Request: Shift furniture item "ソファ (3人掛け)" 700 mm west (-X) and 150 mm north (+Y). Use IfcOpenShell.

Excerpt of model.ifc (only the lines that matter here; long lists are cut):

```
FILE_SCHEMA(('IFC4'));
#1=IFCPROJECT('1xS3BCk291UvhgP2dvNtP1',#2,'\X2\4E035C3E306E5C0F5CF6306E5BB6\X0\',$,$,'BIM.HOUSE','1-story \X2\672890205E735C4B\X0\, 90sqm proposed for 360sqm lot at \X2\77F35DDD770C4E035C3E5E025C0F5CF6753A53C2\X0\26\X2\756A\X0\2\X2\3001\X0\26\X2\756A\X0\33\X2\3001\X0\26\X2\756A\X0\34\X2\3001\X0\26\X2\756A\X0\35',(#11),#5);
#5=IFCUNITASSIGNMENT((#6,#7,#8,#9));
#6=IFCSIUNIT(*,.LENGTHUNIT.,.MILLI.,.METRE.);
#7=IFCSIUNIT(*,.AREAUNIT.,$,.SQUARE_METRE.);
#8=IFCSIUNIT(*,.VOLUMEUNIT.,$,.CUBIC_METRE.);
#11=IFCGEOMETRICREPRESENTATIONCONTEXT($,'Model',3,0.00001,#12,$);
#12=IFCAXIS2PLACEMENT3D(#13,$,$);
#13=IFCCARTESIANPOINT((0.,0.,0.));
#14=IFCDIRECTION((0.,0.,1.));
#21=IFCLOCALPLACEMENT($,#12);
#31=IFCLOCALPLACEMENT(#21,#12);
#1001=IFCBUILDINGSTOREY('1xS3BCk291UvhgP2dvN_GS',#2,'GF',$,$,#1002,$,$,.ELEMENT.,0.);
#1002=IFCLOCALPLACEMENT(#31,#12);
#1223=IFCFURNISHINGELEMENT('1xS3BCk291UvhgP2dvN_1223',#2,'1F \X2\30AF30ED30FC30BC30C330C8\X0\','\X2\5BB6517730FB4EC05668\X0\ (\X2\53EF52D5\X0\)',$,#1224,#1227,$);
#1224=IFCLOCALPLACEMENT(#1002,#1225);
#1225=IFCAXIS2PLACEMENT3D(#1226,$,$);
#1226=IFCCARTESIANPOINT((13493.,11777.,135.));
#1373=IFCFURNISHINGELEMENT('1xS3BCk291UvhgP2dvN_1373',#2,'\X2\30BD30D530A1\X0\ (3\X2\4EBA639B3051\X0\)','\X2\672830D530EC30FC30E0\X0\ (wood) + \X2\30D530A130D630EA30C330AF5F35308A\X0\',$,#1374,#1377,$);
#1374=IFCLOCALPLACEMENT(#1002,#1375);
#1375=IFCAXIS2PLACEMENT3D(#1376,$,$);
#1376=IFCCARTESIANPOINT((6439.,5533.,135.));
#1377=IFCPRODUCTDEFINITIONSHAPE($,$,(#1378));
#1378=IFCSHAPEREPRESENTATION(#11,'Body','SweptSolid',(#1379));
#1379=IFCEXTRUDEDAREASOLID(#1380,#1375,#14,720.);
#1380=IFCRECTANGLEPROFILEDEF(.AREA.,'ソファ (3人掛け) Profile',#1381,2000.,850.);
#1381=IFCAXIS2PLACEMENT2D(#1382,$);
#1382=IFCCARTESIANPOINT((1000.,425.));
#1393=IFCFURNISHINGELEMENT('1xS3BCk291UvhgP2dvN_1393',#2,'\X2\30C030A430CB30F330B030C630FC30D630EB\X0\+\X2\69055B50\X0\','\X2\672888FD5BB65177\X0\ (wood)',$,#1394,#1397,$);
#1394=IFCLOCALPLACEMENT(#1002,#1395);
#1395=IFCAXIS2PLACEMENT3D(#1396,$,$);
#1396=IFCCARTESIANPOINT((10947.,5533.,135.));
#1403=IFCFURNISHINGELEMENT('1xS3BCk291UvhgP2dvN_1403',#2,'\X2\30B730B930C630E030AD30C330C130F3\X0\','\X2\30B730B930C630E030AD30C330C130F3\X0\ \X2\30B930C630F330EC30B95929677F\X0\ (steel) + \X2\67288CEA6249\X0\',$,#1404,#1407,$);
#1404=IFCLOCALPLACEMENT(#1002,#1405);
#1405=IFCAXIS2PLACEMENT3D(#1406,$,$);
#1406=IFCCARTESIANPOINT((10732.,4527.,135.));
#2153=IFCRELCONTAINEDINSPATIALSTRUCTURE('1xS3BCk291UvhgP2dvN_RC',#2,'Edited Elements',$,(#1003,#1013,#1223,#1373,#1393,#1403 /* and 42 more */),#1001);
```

```python
import ifcopenshell
import ifcopenshell.api.geometry
import ifcopenshell.util.placement
import ifcopenshell.util.unit

model = ifcopenshell.open("model.ifc")
unit_scale = ifcopenshell.util.unit.calculate_unit_scale(model)

item = model.by_guid("1xS3BCk291UvhgP2dvN_1373")
matrix = ifcopenshell.util.placement.get_local_placement(item.ObjectPlacement)
matrix[0, 3] -= 0.7 / unit_scale
matrix[1, 3] += 0.15 / unit_scale
ifcopenshell.api.geometry.edit_object_placement(model, product=item, matrix=matrix, is_si=False)

print(ifcopenshell.util.placement.get_local_placement(item.ObjectPlacement).round(3) + 0.0)

model.write("model_updated.ifc")
```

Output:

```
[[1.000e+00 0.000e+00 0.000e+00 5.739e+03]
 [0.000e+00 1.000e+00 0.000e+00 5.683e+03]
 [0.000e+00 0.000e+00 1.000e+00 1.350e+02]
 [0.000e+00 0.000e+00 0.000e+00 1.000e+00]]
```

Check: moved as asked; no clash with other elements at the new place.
